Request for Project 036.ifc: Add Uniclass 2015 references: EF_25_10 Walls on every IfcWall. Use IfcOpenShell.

First a look at what the model holds.

```python
import ifcopenshell

model = ifcopenshell.open("Project 036.ifc")
print(model.schema)
print("classifications:", [c.Name for c in model.by_type("IfcClassification")])
for ifc_class in ("IfcDoor", "IfcRoof", "IfcStair", "IfcWall", "IfcWindow"):
    print(ifc_class, len(model.by_type(ifc_class)))
```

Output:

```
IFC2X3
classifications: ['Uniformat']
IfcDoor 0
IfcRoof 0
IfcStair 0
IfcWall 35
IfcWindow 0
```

```python
import ifcopenshell
import ifcopenshell.api.classification

model = ifcopenshell.open("Project 036.ifc")

# IFC2X3 requires Source and Edition and has no link from the project to the system.
system = model.create_entity("IfcClassification", Source="NBS", Edition="2015", Name="Uniclass 2015")

codes = {
    "IfcWall": ("EF_25_10", "Walls"),
}
for ifc_class, (code, name) in codes.items():
    products = model.by_type(ifc_class)
    ifcopenshell.api.classification.add_reference(
        model, products=products, classification=system, identification=code, name=name
    )
    print(code, len(products))

model.write("Project 036-out.ifc")
```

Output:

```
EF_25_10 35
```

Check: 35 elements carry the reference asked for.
